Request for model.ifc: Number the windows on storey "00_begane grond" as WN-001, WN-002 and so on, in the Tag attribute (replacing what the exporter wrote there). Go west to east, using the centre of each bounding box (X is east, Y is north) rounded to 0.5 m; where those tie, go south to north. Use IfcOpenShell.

First a look at what the model holds.

```python
import ifcopenshell
import ifcopenshell.util.element
import ifcopenshell.util.placement

model = ifcopenshell.open("model.ifc")
print(model.schema)
storey = next(s for s in model.by_type("IfcBuildingStorey") if s.Name == "00_begane grond")
windows = [e for e in ifcopenshell.util.element.get_decomposition(storey) if e.is_a("IfcWindow")]
for e in sorted(windows, key=lambda e: e.id()):
    origin = ifcopenshell.util.placement.get_local_placement(e.ObjectPlacement)[:3, 3]
    print(e.id(), e.Tag, e.Name, origin.round(2) + 0.0, sep=" | ")
```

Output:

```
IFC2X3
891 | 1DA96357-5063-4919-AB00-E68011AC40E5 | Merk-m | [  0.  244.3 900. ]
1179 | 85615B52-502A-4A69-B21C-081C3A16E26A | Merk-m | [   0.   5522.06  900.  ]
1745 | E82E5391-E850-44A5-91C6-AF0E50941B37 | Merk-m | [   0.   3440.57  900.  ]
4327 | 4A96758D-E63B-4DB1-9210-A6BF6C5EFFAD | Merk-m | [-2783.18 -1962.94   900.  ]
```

```python
import ifcopenshell
import ifcopenshell.geom
import ifcopenshell.util.element
import ifcopenshell.util.shape

model = ifcopenshell.open("model.ifc")
settings = ifcopenshell.geom.settings()
settings.set("use-world-coords", True)


def centre(element):
    shape = ifcopenshell.geom.create_shape(settings, element)
    return ifcopenshell.util.shape.get_bbox_centroid(shape.geometry)


storey = next(s for s in model.by_type("IfcBuildingStorey") if s.Name == "00_begane grond")
windows = [e for e in ifcopenshell.util.element.get_decomposition(storey) if e.is_a("IfcWindow")]

# Insertion points can sit at a corner or the storey origin, so sort by the geometry (in metres).
centres = {e: centre(e) for e in windows}
windows.sort(key=lambda e: (round(centres[e][0] / 0.5), centres[e][1]))

for i, e in enumerate(windows, start=1):
    number = f"WN-0{i:02d}"
    e.Tag = number
    print(e.id(), number)

model.write("model_edited.ifc")
```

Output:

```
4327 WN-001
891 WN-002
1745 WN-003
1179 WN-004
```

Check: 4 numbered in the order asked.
